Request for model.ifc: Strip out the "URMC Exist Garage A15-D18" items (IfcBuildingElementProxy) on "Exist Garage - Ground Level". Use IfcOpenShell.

First a look at what the model holds.

```python
import ifcopenshell
import ifcopenshell.util.element

model = ifcopenshell.open("model.ifc")
print(model.schema)
storey = next(s for s in model.by_type("IfcBuildingStorey") if s.Name == "Exist Garage - Ground Level")
proxies = [e for e in ifcopenshell.util.element.get_decomposition(storey) if e.is_a("IfcBuildingElementProxy")]
seen = {}
for e in proxies:
    element_type = ifcopenshell.util.element.get_type(e)
    name = element_type.Name if element_type not in (None, e) else None
    seen[name] = seen.get(name, 0) + 1
for name, count in sorted(seen.items(), key=str):
    print(count, "x", name)
```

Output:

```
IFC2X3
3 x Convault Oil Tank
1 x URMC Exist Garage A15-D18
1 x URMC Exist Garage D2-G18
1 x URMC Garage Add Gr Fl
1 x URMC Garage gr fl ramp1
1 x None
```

```python
import ifcopenshell
import ifcopenshell.api.root
import ifcopenshell.util.element

model = ifcopenshell.open("model.ifc")

storey = next(s for s in model.by_type("IfcBuildingStorey") if s.Name == "Exist Garage - Ground Level")
proxies = [e for e in ifcopenshell.util.element.get_decomposition(storey) if e.is_a("IfcBuildingElementProxy")]
targets = [e for e in proxies if (t := ifcopenshell.util.element.get_type(e)) not in (None, e) and t.Name == "URMC Exist Garage A15-D18"]

for e in targets:
    ifcopenshell.api.root.remove_product(model, product=e)
print(len(targets), "removed")

model.write("model_edited.ifc")
```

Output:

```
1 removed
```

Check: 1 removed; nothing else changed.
